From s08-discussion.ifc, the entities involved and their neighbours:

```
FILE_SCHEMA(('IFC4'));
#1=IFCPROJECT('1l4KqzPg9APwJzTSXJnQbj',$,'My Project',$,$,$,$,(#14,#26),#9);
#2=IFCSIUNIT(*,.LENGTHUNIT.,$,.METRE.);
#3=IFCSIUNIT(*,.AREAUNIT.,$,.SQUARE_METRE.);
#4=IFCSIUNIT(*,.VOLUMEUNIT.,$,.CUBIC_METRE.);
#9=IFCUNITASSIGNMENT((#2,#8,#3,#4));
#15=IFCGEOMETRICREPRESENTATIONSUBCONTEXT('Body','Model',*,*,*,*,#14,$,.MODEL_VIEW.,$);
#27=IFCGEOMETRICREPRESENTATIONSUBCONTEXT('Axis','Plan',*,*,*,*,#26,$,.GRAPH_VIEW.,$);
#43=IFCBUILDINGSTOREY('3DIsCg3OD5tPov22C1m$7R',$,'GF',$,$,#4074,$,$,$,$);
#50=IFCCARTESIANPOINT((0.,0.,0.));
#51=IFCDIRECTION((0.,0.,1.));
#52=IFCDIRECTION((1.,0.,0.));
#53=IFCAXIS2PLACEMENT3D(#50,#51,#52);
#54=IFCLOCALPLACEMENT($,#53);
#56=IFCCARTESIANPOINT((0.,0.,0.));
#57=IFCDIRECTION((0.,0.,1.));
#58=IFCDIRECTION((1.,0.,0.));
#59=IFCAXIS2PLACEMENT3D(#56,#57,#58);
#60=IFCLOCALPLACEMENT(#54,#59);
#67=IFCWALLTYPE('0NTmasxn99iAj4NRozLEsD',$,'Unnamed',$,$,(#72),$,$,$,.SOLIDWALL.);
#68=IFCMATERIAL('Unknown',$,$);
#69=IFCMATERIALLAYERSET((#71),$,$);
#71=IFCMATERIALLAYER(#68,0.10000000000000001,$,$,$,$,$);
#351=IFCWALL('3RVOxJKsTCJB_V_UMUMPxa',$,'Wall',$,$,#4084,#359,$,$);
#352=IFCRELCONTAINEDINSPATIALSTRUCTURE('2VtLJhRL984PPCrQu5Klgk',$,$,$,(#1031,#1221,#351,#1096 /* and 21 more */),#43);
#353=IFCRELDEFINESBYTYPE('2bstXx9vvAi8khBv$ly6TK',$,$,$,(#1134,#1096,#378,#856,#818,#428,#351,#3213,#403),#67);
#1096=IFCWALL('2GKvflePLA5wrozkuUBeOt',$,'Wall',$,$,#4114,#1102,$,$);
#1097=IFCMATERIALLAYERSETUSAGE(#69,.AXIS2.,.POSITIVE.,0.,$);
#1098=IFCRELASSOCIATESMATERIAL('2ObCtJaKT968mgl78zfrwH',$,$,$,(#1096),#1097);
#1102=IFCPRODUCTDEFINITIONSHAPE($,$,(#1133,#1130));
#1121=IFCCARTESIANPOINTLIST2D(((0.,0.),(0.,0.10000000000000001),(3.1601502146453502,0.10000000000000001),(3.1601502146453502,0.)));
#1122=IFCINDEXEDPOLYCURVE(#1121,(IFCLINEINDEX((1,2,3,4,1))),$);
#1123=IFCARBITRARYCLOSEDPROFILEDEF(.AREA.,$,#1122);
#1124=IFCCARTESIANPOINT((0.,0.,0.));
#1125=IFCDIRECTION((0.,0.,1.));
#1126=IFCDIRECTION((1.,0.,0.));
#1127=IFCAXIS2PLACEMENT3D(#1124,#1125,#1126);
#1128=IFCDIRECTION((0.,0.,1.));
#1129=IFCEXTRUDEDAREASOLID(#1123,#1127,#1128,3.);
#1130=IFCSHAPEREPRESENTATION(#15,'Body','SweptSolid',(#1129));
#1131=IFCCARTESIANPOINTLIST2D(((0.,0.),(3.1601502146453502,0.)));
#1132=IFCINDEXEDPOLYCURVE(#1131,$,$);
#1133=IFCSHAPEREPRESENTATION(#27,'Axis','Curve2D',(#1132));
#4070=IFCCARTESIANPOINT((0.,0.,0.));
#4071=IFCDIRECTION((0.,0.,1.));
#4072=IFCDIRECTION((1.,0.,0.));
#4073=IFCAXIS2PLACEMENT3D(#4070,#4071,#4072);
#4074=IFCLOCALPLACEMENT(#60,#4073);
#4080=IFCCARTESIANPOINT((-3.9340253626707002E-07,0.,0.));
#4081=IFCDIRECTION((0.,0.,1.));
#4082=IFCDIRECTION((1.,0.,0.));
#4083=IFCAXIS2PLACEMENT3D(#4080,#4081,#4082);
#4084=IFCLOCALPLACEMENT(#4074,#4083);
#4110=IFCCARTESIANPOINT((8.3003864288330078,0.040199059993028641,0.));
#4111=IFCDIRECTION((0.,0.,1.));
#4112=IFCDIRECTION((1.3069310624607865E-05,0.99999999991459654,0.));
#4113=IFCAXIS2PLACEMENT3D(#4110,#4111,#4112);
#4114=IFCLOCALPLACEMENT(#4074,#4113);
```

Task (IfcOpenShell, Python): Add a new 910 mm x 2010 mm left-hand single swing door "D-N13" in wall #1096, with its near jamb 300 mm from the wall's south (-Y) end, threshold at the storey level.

```python
import numpy as np
import ifcopenshell
import ifcopenshell.api.feature
import ifcopenshell.api.geometry
import ifcopenshell.api.root
import ifcopenshell.api.spatial
import ifcopenshell.geom
import ifcopenshell.util.element
import ifcopenshell.util.placement
import ifcopenshell.util.representation
import ifcopenshell.util.shape
import ifcopenshell.util.unit

model = ifcopenshell.open("s08-discussion.ifc")
unit_scale = ifcopenshell.util.unit.calculate_unit_scale(model)
settings = ifcopenshell.geom.settings()


def volume(element):
    """Net volume in cubic metres, openings subtracted."""
    shape = ifcopenshell.geom.create_shape(settings, element)
    return ifcopenshell.util.shape.get_volume(shape.geometry)


wall = model.by_id(1096)
storey = ifcopenshell.util.element.get_container(wall, ifc_class="IfcBuildingStorey")
context = ifcopenshell.util.representation.get_context(model, "Model", "Body", "MODEL_VIEW")
before = volume(wall)

width, height, from_end, sill = 0.91, 2.01, 0.3, 0.0  # metres

# The wall runs along its own X axis, and the end named is its -X end.
wall_shape = ifcopenshell.geom.create_shape(settings, wall)
x, y, z = ifcopenshell.util.shape.get_vertices(wall_shape.geometry).T
start = x.min() + from_end
face, thickness = float(y.min()), float(y.max() - y.min())
wall_matrix = ifcopenshell.util.placement.get_local_placement(wall.ObjectPlacement)
level = ifcopenshell.util.placement.get_local_placement(storey.ObjectPlacement)[2, 3]


def in_wall(x, y):
    """Placement at x, y metres in the wall's axes, at sill height."""
    matrix = wall_matrix.copy()
    matrix[:, 3] = wall_matrix @ np.array([x / unit_scale, y / unit_scale, 0.0, 1.0])
    matrix[2, 3] = level + sill / unit_scale
    return matrix


# Opening: a box that overshoots both wall faces by 50 mm.
opening = ifcopenshell.api.root.create_entity(model, ifc_class="IfcOpeningElement", predefined_type="OPENING")
box = ifcopenshell.api.geometry.add_wall_representation(
    model, context=context, length=width, height=height, thickness=thickness + 0.1
)
ifcopenshell.api.geometry.assign_representation(model, product=opening, representation=box)
ifcopenshell.api.geometry.edit_object_placement(model, product=opening, matrix=in_wall(start, face - 0.05), is_si=False)
ifcopenshell.api.feature.add_feature(model, feature=opening, element=wall)

door = ifcopenshell.api.root.create_entity(model, ifc_class="IfcDoor", name="D-N13", predefined_type="DOOR")
door.OverallWidth, door.OverallHeight = width / unit_scale, height / unit_scale
door.OperationType = "SINGLE_SWING_LEFT"
body = ifcopenshell.api.geometry.add_door_representation(
    model,
    context=context,
    overall_width=door.OverallWidth,
    overall_height=door.OverallHeight,
    operation_type="SINGLE_SWING_LEFT",
    lining_properties={"LiningDepth": thickness / unit_scale, "ThresholdDepth": thickness / unit_scale},
)
ifcopenshell.api.geometry.assign_representation(model, product=door, representation=body)
ifcopenshell.api.spatial.assign_container(model, products=[door], relating_structure=storey)
ifcopenshell.api.feature.add_filling(model, opening=opening, element=door)

# The lining spans the wall, so the door starts at the wall face.
ifcopenshell.api.geometry.edit_object_placement(model, product=door, matrix=in_wall(start, face), is_si=False)

after = volume(wall)

print(f"wall volume {before:.3f} -> {after:.3f} m3")

model.write("s08-discussion-out.ifc")
```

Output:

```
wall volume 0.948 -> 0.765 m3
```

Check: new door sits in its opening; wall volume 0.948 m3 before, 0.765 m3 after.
